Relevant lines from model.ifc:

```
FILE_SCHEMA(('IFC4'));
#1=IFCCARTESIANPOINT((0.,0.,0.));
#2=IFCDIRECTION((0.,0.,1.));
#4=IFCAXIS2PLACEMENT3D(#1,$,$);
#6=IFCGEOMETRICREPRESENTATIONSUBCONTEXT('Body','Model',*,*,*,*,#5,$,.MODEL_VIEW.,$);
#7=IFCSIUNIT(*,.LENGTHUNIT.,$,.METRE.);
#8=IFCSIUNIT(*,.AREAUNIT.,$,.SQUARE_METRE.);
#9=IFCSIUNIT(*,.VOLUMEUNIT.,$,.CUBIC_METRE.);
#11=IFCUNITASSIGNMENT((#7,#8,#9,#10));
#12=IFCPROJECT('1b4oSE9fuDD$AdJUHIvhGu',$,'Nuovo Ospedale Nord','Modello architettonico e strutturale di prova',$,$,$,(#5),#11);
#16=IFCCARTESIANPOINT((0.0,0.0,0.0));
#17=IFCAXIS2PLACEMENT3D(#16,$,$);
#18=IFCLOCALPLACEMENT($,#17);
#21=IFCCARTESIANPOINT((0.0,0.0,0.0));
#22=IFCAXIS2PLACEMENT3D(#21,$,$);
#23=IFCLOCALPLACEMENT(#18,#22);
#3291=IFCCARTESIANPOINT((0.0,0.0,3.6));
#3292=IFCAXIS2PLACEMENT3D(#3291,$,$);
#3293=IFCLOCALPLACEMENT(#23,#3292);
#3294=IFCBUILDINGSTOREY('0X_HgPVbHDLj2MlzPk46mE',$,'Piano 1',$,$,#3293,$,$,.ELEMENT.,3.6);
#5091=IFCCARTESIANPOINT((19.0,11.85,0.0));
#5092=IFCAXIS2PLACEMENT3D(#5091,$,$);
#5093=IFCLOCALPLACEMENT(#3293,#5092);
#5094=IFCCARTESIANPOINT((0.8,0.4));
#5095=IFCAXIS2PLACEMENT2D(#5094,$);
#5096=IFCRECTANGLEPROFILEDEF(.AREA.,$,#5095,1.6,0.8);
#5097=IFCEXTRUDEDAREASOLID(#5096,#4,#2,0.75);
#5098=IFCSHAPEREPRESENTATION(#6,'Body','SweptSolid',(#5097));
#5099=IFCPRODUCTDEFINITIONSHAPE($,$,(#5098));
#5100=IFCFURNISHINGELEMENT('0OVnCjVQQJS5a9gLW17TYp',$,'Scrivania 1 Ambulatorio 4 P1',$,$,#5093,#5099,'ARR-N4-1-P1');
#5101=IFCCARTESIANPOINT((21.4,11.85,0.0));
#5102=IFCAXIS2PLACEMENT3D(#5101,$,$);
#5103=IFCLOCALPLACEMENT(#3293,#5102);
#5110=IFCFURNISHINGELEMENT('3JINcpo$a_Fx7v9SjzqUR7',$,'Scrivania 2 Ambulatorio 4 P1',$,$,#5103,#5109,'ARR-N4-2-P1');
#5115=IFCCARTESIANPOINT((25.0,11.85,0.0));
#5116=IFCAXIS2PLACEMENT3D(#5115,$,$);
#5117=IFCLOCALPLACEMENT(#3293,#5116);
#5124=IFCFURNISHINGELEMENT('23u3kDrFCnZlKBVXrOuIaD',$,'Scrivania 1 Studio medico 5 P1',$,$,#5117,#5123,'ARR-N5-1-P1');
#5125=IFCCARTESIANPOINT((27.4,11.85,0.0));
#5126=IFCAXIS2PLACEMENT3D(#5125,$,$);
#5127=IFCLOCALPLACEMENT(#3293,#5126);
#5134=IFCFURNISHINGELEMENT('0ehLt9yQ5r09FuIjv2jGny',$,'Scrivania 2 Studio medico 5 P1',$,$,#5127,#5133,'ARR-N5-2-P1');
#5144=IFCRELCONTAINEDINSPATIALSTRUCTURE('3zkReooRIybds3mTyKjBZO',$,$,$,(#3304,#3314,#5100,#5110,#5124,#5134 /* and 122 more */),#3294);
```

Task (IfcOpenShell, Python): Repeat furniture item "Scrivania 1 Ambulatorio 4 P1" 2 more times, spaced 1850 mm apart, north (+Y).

```python
import numpy as np
import ifcopenshell
import ifcopenshell.api.geometry
import ifcopenshell.api.root
import ifcopenshell.util.element
import ifcopenshell.util.placement

model = ifcopenshell.open("model.ifc")

source = model.by_id(5100)
base = ifcopenshell.util.placement.get_local_placement(source.ObjectPlacement)
step = np.array([0.0, 1.0, 0.0]) * 1.85

for i in range(1, 3):
    copy = ifcopenshell.api.root.copy_class(model, product=source)
    copy.Representation = ifcopenshell.util.element.copy_deep(
        model, source.Representation, exclude=["IfcGeometricRepresentationContext", "IfcRepresentationMap"]
    )
    copy.Tag = None
    matrix = base.copy()
    matrix[:3, 3] += i * step
    print("added at", matrix[:3, 3].round(3) + 0.0)
    ifcopenshell.api.geometry.edit_object_placement(model, product=copy, matrix=matrix, is_si=False)

model.write("model-out.ifc")
```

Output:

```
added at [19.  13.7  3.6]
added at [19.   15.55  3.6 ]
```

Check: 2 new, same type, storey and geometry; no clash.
